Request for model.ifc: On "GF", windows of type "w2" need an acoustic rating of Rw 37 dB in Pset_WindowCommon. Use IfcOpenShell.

First a look at what the model holds.

```python
import ifcopenshell
import ifcopenshell.util.element

model = ifcopenshell.open("model.ifc")
print(model.schema)
storey = next(s for s in model.by_type("IfcBuildingStorey") if s.Name == "GF")
windows = [e for e in ifcopenshell.util.element.get_decomposition(storey) if e.is_a("IfcWindow")]
seen = {}
for e in windows:
    element_type = ifcopenshell.util.element.get_type(e)
    key = (element_type.Name if element_type != e and element_type else None, ifcopenshell.util.element.get_pset(e, "Pset_WindowCommon", "AcousticRating"))
    seen[key] = seen.get(key, 0) + 1
for (name, value), count in sorted(seen.items(), key=str):
    print(count, "x", name, "|", value)
```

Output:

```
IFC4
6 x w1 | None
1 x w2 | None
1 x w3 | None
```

```python
import ifcopenshell
import ifcopenshell.api.pset
import ifcopenshell.util.element

model = ifcopenshell.open("model.ifc")

storey = next(s for s in model.by_type("IfcBuildingStorey") if s.Name == "GF")
windows = [e for e in ifcopenshell.util.element.get_decomposition(storey) if e.is_a("IfcWindow")]

count = 0
for e in windows:
    element_type = ifcopenshell.util.element.get_type(e)
    if element_type in (None, e) or element_type.Name != "w2":
        continue
    # add_pset returns the element's existing set when there is one.
    pset = ifcopenshell.api.pset.add_pset(model, product=e, name="Pset_WindowCommon")
    ifcopenshell.api.pset.edit_pset(model, pset=pset, properties={"AcousticRating": "Rw 37 dB"})
    count += 1

print(count, "windows updated")

model.write("model_edited.ifc")
```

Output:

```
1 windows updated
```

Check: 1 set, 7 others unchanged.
